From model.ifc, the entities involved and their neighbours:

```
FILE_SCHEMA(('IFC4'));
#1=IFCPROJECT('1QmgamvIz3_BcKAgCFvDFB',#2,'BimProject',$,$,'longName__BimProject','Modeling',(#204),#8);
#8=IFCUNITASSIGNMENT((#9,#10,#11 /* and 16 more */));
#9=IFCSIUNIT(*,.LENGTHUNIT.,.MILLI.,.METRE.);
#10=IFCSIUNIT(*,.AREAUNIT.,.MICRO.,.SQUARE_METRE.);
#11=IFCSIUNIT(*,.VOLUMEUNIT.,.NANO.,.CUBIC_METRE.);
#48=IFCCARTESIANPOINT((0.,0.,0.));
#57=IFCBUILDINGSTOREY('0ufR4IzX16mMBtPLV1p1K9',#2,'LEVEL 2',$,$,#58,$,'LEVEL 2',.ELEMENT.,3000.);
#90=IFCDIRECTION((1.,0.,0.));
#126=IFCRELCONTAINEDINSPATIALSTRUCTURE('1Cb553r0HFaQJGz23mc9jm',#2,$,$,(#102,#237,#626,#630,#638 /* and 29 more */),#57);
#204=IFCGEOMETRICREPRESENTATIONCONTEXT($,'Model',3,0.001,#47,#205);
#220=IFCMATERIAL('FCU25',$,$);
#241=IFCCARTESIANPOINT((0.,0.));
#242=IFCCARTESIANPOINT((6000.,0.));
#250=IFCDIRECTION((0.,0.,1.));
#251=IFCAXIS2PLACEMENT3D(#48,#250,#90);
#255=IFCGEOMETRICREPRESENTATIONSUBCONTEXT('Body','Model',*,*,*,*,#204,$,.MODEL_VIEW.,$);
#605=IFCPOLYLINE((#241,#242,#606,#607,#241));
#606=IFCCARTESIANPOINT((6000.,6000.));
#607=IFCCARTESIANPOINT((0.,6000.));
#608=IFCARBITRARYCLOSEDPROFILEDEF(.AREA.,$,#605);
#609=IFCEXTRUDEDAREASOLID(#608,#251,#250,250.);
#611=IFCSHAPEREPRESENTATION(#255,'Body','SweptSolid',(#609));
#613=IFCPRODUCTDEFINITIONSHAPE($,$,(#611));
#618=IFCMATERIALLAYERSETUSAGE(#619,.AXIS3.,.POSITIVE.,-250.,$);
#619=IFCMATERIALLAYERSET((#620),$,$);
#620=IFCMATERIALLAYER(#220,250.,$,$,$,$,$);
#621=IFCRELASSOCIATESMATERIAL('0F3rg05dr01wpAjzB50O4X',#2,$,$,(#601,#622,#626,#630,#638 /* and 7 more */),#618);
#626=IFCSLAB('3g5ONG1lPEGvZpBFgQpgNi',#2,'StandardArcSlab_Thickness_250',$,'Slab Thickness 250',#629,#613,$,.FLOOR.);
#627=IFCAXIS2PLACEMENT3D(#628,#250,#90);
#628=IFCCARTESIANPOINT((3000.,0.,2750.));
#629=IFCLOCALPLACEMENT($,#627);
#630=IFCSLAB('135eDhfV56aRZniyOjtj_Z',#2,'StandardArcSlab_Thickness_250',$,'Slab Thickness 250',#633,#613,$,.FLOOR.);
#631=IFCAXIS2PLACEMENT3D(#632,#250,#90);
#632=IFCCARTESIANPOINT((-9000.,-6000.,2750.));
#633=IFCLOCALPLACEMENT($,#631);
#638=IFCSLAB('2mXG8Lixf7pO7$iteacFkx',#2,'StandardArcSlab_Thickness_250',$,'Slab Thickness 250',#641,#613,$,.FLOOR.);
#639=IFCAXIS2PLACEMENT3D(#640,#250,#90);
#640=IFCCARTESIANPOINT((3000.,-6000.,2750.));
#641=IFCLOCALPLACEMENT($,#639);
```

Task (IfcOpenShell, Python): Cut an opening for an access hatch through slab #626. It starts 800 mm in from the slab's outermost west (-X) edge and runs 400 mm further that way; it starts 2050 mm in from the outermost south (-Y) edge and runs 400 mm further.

```python
import numpy as np
import ifcopenshell
import ifcopenshell.api.feature
import ifcopenshell.api.geometry
import ifcopenshell.api.root
import ifcopenshell.geom
import ifcopenshell.util.placement
import ifcopenshell.util.representation
import ifcopenshell.util.shape
import ifcopenshell.util.unit

model = ifcopenshell.open("model.ifc")
unit_scale = ifcopenshell.util.unit.calculate_unit_scale(model)
settings = ifcopenshell.geom.settings()


def volume(element):
    """Net volume in cubic metres, openings subtracted."""
    shape = ifcopenshell.geom.create_shape(settings, element)
    return ifcopenshell.util.shape.get_volume(shape.geometry)


slab = model.by_guid("3g5ONG1lPEGvZpBFgQpgNi")
before = volume(slab)

# Extent in the slab's own axes, in metres. The edges named are its -X and -Y sides.
slab_shape = ifcopenshell.geom.create_shape(settings, slab)
vertices = ifcopenshell.util.shape.get_vertices(slab_shape.geometry)
x_min, y_min, bottom = vertices.min(axis=0)
top = vertices[:, 2].max()

opening = ifcopenshell.api.root.create_entity(model, ifc_class="IfcOpeningElement", name="Access hatch opening", predefined_type="OPENING")
context = ifcopenshell.util.representation.get_context(model, "Model", "Body", "MODEL_VIEW")
width, depth = 0.4, 0.4
outline = [(0.0, 0.0), (width, 0.0), (width, depth), (0.0, depth), (0.0, 0.0)]
# Overshoot both faces by 50 mm so the cut is clean.
shape = ifcopenshell.api.geometry.add_slab_representation(
    model, context=context, depth=top - bottom + 0.1, polyline=outline
)
ifcopenshell.api.geometry.assign_representation(model, product=opening, representation=shape)

matrix = ifcopenshell.util.placement.get_local_placement(slab.ObjectPlacement)
matrix[:, 3] = matrix @ np.append(np.array([x_min + 0.8, y_min + 2.05, bottom - 0.05]) / unit_scale, 1.0)
ifcopenshell.api.geometry.edit_object_placement(model, product=opening, matrix=matrix, is_si=False)
ifcopenshell.api.feature.add_feature(model, feature=opening, element=slab)

after = volume(slab)

print(f"slab volume {before:.3f} -> {after:.3f} m3")

model.write("model_edited.ifc")
```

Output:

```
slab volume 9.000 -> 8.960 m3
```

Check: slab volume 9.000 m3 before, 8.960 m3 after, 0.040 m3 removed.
